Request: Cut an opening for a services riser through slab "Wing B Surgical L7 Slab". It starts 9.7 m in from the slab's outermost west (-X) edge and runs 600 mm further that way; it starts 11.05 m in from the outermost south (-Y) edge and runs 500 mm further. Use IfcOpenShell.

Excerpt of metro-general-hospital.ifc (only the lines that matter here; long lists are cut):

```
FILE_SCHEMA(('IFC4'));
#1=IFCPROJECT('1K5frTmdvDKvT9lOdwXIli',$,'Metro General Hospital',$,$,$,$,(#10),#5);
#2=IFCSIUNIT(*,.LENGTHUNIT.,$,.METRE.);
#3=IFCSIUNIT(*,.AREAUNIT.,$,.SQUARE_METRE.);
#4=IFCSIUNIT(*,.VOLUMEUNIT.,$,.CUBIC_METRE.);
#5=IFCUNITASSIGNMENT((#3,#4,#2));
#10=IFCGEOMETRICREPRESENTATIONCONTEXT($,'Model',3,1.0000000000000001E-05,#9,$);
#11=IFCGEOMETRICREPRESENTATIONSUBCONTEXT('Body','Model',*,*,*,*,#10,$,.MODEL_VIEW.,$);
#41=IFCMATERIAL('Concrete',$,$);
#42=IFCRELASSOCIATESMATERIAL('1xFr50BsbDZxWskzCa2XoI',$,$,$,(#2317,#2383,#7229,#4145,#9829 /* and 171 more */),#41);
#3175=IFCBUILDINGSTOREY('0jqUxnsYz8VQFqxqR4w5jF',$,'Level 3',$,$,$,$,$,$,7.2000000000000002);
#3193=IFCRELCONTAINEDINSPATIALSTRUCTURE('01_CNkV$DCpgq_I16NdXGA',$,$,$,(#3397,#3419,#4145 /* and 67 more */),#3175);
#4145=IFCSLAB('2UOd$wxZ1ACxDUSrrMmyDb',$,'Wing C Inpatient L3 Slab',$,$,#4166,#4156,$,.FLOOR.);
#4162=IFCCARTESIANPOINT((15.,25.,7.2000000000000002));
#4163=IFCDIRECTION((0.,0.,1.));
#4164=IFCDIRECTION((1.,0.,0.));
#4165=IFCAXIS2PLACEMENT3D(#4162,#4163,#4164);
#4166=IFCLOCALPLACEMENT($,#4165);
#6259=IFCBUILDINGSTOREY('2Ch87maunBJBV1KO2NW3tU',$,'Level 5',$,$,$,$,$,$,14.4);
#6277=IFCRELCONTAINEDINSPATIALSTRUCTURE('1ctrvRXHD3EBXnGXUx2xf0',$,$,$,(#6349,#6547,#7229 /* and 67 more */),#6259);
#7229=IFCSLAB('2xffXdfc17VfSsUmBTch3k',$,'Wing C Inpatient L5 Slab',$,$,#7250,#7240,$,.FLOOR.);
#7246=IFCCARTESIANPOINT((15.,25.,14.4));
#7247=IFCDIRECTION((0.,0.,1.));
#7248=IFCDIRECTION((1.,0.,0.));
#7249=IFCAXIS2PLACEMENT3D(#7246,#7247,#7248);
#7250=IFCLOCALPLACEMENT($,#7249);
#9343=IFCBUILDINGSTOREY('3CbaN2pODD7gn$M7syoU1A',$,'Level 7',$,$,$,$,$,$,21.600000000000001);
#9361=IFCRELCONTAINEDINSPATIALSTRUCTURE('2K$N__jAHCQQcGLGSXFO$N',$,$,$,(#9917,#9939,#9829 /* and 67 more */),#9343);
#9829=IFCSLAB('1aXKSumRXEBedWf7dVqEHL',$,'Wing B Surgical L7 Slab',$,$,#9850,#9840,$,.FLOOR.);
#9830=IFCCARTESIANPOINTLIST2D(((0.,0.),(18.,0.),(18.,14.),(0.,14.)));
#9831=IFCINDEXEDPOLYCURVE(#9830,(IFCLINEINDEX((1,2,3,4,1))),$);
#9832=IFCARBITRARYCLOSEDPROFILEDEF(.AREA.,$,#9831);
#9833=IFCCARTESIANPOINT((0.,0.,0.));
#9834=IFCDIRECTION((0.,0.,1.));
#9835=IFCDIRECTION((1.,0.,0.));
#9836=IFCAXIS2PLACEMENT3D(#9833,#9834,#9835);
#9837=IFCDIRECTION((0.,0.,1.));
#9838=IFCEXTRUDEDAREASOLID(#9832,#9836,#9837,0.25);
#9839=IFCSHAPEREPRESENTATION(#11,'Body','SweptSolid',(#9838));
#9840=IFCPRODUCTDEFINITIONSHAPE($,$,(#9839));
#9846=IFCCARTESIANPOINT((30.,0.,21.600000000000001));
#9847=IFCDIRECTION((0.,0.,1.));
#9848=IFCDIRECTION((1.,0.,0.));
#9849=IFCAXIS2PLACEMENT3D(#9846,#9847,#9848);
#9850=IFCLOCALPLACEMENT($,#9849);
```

```python
import numpy as np
import ifcopenshell
import ifcopenshell.api.feature
import ifcopenshell.api.geometry
import ifcopenshell.api.root
import ifcopenshell.geom
import ifcopenshell.util.placement
import ifcopenshell.util.representation
import ifcopenshell.util.shape
import ifcopenshell.util.unit

model = ifcopenshell.open("metro-general-hospital.ifc")
unit_scale = ifcopenshell.util.unit.calculate_unit_scale(model)
settings = ifcopenshell.geom.settings()


def volume(element):
    """Net volume in cubic metres, openings subtracted."""
    shape = ifcopenshell.geom.create_shape(settings, element)
    return ifcopenshell.util.shape.get_volume(shape.geometry)


slab = model.by_guid("1aXKSumRXEBedWf7dVqEHL")
before = volume(slab)

# Extent in the slab's own axes, in metres. The edges named are its -X and -Y sides.
slab_shape = ifcopenshell.geom.create_shape(settings, slab)
vertices = ifcopenshell.util.shape.get_vertices(slab_shape.geometry)
x_min, y_min, bottom = vertices.min(axis=0)
top = vertices[:, 2].max()

opening = ifcopenshell.api.root.create_entity(model, ifc_class="IfcOpeningElement", name="Services riser opening", predefined_type="OPENING")
context = ifcopenshell.util.representation.get_context(model, "Model", "Body", "MODEL_VIEW")
width, depth = 0.6, 0.5
outline = [(0.0, 0.0), (width, 0.0), (width, depth), (0.0, depth), (0.0, 0.0)]
# Overshoot both faces by 50 mm so the cut is clean.
shape = ifcopenshell.api.geometry.add_slab_representation(
    model, context=context, depth=top - bottom + 0.1, polyline=outline
)
ifcopenshell.api.geometry.assign_representation(model, product=opening, representation=shape)

matrix = ifcopenshell.util.placement.get_local_placement(slab.ObjectPlacement)
matrix[:, 3] = matrix @ np.append(np.array([x_min + 9.7, y_min + 11.05, bottom - 0.05]) / unit_scale, 1.0)
ifcopenshell.api.geometry.edit_object_placement(model, product=opening, matrix=matrix, is_si=False)
ifcopenshell.api.feature.add_feature(model, feature=opening, element=slab)

after = volume(slab)

print(f"slab volume {before:.3f} -> {after:.3f} m3")

model.write("metro-general-hospital_rev.ifc")
```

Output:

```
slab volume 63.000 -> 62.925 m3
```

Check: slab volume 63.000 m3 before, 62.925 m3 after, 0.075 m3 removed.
